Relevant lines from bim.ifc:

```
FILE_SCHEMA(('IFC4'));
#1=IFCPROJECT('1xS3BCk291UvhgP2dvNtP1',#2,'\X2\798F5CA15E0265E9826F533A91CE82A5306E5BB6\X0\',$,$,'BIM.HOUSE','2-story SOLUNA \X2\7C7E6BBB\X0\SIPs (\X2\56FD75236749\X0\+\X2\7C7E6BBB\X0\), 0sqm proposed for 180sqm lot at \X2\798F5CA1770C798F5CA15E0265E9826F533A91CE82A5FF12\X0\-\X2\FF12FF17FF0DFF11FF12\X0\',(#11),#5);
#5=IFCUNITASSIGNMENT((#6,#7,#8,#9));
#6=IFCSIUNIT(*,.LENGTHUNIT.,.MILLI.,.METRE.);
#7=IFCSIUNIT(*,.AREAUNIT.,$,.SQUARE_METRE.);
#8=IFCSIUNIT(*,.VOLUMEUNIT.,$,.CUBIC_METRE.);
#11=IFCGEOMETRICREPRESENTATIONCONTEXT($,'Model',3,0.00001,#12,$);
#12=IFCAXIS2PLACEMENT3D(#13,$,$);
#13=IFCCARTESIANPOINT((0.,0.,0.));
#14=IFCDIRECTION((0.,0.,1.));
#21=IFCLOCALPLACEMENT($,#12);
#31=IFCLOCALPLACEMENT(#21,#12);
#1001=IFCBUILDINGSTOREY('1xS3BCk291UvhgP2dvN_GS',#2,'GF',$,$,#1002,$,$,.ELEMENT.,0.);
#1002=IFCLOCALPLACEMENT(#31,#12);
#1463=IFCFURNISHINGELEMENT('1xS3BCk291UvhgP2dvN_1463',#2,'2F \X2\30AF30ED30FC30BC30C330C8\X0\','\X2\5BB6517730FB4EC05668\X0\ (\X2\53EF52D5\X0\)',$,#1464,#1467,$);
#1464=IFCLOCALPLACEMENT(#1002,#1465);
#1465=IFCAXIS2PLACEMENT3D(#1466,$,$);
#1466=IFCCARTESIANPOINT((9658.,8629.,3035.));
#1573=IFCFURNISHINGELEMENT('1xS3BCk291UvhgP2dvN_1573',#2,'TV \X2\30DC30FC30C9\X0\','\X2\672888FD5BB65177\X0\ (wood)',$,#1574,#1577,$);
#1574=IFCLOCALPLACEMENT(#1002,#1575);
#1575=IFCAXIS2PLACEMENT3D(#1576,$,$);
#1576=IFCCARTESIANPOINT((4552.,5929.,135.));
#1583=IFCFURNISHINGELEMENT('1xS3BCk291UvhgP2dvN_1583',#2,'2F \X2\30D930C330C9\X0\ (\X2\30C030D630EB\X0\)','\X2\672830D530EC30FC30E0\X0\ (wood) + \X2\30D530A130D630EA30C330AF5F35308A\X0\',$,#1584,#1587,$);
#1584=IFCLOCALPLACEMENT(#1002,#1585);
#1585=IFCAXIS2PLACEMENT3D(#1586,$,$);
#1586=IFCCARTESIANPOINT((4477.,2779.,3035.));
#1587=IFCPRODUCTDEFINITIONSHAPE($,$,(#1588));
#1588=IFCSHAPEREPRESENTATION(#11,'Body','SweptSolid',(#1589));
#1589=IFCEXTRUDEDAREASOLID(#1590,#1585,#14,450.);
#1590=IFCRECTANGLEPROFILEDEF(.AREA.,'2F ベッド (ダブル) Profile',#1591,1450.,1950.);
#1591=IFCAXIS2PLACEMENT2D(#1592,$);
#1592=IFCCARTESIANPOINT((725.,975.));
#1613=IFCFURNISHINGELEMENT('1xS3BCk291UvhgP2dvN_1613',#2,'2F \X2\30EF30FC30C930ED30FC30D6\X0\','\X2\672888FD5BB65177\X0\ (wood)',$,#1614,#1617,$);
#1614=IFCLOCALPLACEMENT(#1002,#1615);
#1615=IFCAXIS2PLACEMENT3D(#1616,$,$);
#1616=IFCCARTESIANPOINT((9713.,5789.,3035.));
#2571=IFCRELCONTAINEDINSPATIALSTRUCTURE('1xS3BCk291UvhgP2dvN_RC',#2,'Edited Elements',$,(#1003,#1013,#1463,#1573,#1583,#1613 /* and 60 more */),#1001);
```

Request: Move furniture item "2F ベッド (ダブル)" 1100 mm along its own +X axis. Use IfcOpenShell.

```python
import ifcopenshell
import ifcopenshell.api.geometry
import ifcopenshell.util.placement
import ifcopenshell.util.unit

model = ifcopenshell.open("bim.ifc")
unit_scale = ifcopenshell.util.unit.calculate_unit_scale(model)

item = model.by_id(1583)
matrix = ifcopenshell.util.placement.get_local_placement(item.ObjectPlacement)
matrix[:3, 3] += matrix[:3, 0] * 1.1 / unit_scale
ifcopenshell.api.geometry.edit_object_placement(model, product=item, matrix=matrix, is_si=False)

print(ifcopenshell.util.placement.get_local_placement(item.ObjectPlacement).round(3) + 0.0)

model.write("bim_updated.ifc")
```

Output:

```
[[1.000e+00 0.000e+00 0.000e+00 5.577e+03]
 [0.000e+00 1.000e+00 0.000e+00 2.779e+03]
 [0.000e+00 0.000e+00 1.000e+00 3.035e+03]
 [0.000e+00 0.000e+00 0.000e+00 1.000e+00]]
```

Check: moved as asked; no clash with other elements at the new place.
